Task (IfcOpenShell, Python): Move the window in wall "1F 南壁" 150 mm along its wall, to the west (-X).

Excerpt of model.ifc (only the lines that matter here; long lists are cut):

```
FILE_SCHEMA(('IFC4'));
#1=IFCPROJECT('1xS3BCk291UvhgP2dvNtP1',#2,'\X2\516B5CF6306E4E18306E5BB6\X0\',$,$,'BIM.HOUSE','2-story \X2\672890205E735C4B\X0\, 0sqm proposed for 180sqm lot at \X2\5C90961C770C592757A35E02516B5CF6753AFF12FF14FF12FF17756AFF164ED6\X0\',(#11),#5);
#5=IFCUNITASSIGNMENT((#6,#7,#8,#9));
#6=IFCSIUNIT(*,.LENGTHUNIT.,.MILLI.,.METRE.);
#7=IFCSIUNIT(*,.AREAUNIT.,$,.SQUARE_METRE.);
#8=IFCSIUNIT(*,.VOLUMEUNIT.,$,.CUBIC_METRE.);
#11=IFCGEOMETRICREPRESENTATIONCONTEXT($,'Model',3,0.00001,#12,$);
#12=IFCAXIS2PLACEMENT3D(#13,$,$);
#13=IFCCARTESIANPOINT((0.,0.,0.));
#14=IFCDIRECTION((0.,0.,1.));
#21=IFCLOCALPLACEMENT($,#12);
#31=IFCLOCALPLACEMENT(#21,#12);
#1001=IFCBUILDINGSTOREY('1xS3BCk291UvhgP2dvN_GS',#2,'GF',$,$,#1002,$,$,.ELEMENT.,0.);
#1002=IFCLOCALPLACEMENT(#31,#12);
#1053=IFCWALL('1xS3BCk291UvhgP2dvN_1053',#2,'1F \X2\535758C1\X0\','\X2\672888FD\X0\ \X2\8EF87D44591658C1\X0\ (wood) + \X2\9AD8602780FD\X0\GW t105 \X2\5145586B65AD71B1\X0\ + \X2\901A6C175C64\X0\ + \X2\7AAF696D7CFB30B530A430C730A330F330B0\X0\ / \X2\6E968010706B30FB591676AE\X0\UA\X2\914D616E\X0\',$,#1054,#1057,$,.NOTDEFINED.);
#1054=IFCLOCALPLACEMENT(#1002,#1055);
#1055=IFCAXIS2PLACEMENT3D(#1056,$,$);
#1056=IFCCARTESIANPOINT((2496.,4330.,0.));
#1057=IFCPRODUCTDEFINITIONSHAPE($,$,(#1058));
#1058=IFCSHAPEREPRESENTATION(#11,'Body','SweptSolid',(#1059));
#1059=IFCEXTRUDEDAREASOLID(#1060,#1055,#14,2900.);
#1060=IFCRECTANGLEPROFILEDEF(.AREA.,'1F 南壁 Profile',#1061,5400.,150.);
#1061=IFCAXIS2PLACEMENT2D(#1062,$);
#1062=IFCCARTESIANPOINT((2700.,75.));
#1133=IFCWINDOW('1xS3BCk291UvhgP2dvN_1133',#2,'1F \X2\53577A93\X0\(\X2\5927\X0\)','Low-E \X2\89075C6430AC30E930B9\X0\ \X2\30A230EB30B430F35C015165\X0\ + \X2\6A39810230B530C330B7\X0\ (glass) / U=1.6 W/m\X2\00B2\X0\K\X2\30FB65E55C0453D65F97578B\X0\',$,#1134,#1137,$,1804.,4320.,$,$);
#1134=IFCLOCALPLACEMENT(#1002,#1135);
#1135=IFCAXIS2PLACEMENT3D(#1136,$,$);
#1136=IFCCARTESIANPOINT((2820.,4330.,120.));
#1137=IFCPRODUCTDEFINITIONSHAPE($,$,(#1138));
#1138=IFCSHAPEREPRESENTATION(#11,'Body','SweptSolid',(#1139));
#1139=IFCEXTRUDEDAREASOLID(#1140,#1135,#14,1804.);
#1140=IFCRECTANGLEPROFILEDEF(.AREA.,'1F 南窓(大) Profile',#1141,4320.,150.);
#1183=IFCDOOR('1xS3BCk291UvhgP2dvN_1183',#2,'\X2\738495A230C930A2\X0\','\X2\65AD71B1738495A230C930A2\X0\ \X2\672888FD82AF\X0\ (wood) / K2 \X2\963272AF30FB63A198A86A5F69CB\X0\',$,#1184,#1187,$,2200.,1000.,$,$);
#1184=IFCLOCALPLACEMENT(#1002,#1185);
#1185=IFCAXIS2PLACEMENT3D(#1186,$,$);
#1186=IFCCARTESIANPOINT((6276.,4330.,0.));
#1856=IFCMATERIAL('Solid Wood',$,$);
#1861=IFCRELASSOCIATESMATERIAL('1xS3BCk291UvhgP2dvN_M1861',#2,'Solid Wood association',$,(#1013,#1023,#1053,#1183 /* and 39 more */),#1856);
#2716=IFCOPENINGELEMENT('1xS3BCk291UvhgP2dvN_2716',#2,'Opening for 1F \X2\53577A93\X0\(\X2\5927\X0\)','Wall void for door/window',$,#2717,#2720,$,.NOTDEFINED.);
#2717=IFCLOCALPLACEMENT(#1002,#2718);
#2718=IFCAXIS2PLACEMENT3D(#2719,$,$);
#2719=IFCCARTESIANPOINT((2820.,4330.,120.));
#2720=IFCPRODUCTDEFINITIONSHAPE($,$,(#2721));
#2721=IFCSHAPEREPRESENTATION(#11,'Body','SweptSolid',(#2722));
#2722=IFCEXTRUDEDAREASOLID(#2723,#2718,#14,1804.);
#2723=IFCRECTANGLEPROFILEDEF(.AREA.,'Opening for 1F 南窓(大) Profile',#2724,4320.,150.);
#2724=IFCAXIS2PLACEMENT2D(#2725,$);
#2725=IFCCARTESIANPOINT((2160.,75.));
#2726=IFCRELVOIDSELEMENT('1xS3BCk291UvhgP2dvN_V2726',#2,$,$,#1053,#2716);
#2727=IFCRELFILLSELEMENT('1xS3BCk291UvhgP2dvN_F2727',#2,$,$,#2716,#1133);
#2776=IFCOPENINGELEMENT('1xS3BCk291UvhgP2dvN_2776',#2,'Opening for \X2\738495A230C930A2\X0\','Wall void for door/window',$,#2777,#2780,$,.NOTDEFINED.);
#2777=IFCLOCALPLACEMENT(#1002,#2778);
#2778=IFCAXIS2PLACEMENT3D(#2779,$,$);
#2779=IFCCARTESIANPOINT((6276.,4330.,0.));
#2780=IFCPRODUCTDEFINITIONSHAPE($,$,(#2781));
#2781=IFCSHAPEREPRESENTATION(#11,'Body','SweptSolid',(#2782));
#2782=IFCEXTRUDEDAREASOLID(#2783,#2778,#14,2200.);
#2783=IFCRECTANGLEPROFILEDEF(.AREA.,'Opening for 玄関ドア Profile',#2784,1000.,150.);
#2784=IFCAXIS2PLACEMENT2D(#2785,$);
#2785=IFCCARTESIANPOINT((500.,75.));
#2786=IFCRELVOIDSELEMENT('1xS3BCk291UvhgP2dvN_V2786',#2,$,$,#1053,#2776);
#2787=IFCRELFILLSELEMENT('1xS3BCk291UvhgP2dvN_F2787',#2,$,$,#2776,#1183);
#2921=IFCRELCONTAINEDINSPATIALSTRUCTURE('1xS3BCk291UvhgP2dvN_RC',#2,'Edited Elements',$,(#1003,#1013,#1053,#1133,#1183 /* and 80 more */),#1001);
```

```python
import ifcopenshell
import ifcopenshell.api.geometry
import ifcopenshell.util.placement

model = ifcopenshell.open("model.ifc")

window = model.by_id(1133)
opening = window.FillsVoids[0].RelatingOpeningElement
wall = opening.VoidsElements[0].RelatingBuildingElement

wall_matrix = ifcopenshell.util.placement.get_local_placement(wall.ObjectPlacement)
shift = wall_matrix[:3, 0] * -150.0
before = ifcopenshell.util.placement.get_local_placement(window.ObjectPlacement)[:3, 3].copy()

# The window is not placed relative to its opening, so move both.
for product in (opening, window):
    matrix = ifcopenshell.util.placement.get_local_placement(product.ObjectPlacement)
    matrix[:3, 3] += shift
    ifcopenshell.api.geometry.edit_object_placement(model, product=product, matrix=matrix, is_si=False)

after = ifcopenshell.util.placement.get_local_placement(window.ObjectPlacement)[:3, 3]
print("window moved by", (after - before).round(3) + 0.0)

model.write("model_v2.ifc")
```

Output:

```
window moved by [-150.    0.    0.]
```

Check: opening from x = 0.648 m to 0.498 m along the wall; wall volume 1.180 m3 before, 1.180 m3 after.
